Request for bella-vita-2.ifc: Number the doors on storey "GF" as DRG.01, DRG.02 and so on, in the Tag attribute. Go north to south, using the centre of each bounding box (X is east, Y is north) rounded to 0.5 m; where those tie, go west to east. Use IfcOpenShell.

First a look at what the model holds.

```python
import ifcopenshell
import ifcopenshell.util.element
import ifcopenshell.util.placement

model = ifcopenshell.open("bella-vita-2.ifc")
print(model.schema)
storey = next(s for s in model.by_type("IfcBuildingStorey") if s.Name == "GF")
doors = [e for e in ifcopenshell.util.element.get_decomposition(storey) if e.is_a("IfcDoor")]
for e in sorted(doors, key=lambda e: e.id()):
    origin = ifcopenshell.util.placement.get_local_placement(e.ObjectPlacement)[:3, 3]
    print(e.id(), e.Tag, e.Name, origin.round(2) + 0.0, sep=" | ")
```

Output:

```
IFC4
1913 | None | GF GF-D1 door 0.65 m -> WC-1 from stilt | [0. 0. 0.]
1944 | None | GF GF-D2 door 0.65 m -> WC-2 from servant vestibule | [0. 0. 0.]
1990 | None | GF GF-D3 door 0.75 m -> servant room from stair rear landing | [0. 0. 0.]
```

```python
import ifcopenshell
import ifcopenshell.geom
import ifcopenshell.util.element
import ifcopenshell.util.shape

model = ifcopenshell.open("bella-vita-2.ifc")
settings = ifcopenshell.geom.settings()
settings.set("use-world-coords", True)


def centre(element):
    shape = ifcopenshell.geom.create_shape(settings, element)
    return ifcopenshell.util.shape.get_bbox_centroid(shape.geometry)


storey = next(s for s in model.by_type("IfcBuildingStorey") if s.Name == "GF")
doors = [e for e in ifcopenshell.util.element.get_decomposition(storey) if e.is_a("IfcDoor")]

# Insertion points can sit at a corner or the storey origin, so sort by the geometry (in metres).
centres = {e: centre(e) for e in doors}
doors.sort(key=lambda e: (-round(centres[e][1] / 0.5), centres[e][0]))

for i, e in enumerate(doors, start=1):
    number = f"DRG.{i:02d}"
    e.Tag = number
    print(e.id(), number)

model.write("bella-vita-2-out.ifc")
```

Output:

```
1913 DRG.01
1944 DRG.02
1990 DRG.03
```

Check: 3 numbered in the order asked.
